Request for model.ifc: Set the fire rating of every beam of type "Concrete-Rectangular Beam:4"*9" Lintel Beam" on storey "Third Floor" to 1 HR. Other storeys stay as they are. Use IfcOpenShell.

First a look at what the model holds.

```python
import ifcopenshell
import ifcopenshell.util.element

model = ifcopenshell.open("model.ifc")
print(model.schema)
storey = next(s for s in model.by_type("IfcBuildingStorey") if s.Name == "Third Floor")
beams = [e for e in ifcopenshell.util.element.get_decomposition(storey) if e.is_a("IfcBeam")]
seen = {}
for e in beams:
    element_type = ifcopenshell.util.element.get_type(e)
    key = (element_type.Name if element_type != e and element_type else None, ifcopenshell.util.element.get_pset(e, "Pset_BeamCommon", "FireRating"))
    seen[key] = seen.get(key, 0) + 1
for (name, value), count in sorted(seen.items(), key=str):
    print(count, "x", name, "|", value)
```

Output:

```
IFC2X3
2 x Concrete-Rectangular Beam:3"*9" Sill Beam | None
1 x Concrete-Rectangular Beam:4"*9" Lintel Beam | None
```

```python
import ifcopenshell
import ifcopenshell.api.pset
import ifcopenshell.util.element

model = ifcopenshell.open("model.ifc")

storey = next(s for s in model.by_type("IfcBuildingStorey") if s.Name == "Third Floor")
beams = [e for e in ifcopenshell.util.element.get_decomposition(storey) if e.is_a("IfcBeam")]

count = 0
for e in beams:
    element_type = ifcopenshell.util.element.get_type(e)
    if element_type in (None, e) or element_type.Name != 'Concrete-Rectangular Beam:4"*9" Lintel Beam':
        continue
    # add_pset returns the element's existing set when there is one.
    pset = ifcopenshell.api.pset.add_pset(model, product=e, name="Pset_BeamCommon")
    ifcopenshell.api.pset.edit_pset(model, pset=pset, properties={"FireRating": "1 HR"})
    count += 1

print(count, "beams updated")

model.write("model_rev.ifc")
```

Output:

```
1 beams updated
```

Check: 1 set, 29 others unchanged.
